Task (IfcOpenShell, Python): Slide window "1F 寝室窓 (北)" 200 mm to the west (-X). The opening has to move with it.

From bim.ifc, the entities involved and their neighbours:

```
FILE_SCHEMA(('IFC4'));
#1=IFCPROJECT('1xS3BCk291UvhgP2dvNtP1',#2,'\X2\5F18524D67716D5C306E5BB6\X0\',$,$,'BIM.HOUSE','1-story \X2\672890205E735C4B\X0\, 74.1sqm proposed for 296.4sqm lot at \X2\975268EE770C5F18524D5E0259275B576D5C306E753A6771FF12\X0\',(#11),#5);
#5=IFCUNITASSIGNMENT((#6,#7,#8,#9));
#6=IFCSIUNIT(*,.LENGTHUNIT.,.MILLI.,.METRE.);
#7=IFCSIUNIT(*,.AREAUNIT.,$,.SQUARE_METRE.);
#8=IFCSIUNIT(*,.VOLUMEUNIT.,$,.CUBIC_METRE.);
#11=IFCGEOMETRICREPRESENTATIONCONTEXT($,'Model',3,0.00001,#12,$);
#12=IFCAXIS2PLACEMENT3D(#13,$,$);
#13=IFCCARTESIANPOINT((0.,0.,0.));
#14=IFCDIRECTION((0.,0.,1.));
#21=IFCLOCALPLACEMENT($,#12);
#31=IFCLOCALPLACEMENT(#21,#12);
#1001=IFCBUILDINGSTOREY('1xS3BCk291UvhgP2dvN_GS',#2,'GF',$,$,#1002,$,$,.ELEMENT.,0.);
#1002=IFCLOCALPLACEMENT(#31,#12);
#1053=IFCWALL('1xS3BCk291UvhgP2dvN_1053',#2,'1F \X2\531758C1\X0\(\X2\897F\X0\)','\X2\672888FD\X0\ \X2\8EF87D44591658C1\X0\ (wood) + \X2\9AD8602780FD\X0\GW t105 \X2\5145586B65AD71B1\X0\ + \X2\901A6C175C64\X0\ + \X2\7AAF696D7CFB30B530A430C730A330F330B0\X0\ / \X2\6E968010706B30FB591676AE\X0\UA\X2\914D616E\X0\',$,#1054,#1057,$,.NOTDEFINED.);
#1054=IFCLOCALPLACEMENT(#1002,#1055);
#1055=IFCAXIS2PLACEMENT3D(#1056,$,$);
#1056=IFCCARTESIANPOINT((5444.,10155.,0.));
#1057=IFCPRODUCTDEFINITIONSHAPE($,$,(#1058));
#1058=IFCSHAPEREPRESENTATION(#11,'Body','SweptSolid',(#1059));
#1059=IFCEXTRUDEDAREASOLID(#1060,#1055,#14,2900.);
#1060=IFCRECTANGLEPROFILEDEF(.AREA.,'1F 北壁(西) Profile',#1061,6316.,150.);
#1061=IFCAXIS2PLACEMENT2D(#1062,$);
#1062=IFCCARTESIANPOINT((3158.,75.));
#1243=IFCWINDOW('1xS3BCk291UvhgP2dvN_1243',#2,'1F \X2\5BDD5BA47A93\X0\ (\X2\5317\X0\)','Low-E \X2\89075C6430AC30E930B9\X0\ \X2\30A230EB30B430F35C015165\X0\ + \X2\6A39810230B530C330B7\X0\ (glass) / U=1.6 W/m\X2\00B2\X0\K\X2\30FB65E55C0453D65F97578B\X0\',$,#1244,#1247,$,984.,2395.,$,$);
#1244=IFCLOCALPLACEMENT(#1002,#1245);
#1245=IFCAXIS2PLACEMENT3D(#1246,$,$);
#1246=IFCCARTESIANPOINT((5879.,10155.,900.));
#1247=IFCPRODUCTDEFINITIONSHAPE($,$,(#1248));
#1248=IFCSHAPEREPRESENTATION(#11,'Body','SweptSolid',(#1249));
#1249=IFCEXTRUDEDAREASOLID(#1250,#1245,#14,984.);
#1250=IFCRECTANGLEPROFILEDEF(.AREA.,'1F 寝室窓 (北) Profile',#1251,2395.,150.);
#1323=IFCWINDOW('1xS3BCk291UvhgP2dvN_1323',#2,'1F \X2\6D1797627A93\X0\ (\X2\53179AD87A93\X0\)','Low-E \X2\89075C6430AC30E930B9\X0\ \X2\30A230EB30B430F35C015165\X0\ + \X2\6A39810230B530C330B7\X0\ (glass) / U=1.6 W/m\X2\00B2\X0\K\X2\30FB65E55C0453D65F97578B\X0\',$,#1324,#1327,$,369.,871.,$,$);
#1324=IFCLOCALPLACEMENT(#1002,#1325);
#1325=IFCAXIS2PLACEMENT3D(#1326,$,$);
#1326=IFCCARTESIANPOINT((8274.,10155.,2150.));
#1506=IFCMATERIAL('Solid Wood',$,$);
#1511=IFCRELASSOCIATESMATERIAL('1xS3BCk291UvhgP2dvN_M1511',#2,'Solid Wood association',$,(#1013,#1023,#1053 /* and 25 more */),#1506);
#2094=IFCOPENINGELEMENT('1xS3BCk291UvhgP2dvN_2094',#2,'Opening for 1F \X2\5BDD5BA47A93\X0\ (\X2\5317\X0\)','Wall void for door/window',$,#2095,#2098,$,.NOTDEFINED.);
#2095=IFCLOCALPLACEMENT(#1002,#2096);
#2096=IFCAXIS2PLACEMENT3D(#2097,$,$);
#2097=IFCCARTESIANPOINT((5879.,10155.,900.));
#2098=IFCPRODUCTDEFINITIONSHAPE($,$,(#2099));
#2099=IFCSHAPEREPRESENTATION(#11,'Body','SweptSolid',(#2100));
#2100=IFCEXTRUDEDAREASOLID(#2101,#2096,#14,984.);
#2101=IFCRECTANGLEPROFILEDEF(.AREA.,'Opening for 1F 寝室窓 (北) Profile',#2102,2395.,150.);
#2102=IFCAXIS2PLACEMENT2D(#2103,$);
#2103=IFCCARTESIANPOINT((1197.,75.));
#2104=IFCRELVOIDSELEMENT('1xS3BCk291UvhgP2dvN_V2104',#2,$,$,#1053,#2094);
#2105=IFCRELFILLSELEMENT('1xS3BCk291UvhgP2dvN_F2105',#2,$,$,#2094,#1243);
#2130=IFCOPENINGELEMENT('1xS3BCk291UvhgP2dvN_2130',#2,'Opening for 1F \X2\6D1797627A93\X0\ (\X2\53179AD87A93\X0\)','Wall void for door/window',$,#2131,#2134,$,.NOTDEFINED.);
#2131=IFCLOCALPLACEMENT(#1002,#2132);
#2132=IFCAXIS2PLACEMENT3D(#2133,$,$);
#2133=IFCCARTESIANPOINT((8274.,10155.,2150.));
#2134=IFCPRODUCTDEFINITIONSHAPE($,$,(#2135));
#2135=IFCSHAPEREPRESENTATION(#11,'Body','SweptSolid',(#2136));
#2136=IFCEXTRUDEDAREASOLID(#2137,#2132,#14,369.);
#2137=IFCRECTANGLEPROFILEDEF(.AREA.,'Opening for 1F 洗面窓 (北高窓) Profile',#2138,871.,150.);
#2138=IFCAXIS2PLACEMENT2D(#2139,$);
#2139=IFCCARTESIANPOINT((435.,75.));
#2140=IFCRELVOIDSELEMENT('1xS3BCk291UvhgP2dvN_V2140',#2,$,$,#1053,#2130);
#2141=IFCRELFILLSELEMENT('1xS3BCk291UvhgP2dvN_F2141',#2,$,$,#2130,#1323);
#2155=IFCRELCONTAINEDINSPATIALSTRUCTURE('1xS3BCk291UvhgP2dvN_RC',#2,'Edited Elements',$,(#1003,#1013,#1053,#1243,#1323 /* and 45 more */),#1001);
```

```python
import ifcopenshell
import ifcopenshell.api.geometry
import ifcopenshell.util.placement
import ifcopenshell.util.unit

model = ifcopenshell.open("bim.ifc")
unit_scale = ifcopenshell.util.unit.calculate_unit_scale(model)

window = model.by_guid("1xS3BCk291UvhgP2dvN_1243")
opening = window.FillsVoids[0].RelatingOpeningElement
wall = opening.VoidsElements[0].RelatingBuildingElement

wall_matrix = ifcopenshell.util.placement.get_local_placement(wall.ObjectPlacement)
shift = wall_matrix[:3, 0] * -0.2 / unit_scale
before = ifcopenshell.util.placement.get_local_placement(window.ObjectPlacement)[:3, 3].copy()

# The window is not placed relative to its opening, so move both.
for product in (opening, window):
    matrix = ifcopenshell.util.placement.get_local_placement(product.ObjectPlacement)
    matrix[:3, 3] += shift
    ifcopenshell.api.geometry.edit_object_placement(model, product=product, matrix=matrix, is_si=False)

after = ifcopenshell.util.placement.get_local_placement(window.ObjectPlacement)[:3, 3]
print("window moved by", (after - before).round(3) + 0.0)

model.write("bim-out.ifc")
```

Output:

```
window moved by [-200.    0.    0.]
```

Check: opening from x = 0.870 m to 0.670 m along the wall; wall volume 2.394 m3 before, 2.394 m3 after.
